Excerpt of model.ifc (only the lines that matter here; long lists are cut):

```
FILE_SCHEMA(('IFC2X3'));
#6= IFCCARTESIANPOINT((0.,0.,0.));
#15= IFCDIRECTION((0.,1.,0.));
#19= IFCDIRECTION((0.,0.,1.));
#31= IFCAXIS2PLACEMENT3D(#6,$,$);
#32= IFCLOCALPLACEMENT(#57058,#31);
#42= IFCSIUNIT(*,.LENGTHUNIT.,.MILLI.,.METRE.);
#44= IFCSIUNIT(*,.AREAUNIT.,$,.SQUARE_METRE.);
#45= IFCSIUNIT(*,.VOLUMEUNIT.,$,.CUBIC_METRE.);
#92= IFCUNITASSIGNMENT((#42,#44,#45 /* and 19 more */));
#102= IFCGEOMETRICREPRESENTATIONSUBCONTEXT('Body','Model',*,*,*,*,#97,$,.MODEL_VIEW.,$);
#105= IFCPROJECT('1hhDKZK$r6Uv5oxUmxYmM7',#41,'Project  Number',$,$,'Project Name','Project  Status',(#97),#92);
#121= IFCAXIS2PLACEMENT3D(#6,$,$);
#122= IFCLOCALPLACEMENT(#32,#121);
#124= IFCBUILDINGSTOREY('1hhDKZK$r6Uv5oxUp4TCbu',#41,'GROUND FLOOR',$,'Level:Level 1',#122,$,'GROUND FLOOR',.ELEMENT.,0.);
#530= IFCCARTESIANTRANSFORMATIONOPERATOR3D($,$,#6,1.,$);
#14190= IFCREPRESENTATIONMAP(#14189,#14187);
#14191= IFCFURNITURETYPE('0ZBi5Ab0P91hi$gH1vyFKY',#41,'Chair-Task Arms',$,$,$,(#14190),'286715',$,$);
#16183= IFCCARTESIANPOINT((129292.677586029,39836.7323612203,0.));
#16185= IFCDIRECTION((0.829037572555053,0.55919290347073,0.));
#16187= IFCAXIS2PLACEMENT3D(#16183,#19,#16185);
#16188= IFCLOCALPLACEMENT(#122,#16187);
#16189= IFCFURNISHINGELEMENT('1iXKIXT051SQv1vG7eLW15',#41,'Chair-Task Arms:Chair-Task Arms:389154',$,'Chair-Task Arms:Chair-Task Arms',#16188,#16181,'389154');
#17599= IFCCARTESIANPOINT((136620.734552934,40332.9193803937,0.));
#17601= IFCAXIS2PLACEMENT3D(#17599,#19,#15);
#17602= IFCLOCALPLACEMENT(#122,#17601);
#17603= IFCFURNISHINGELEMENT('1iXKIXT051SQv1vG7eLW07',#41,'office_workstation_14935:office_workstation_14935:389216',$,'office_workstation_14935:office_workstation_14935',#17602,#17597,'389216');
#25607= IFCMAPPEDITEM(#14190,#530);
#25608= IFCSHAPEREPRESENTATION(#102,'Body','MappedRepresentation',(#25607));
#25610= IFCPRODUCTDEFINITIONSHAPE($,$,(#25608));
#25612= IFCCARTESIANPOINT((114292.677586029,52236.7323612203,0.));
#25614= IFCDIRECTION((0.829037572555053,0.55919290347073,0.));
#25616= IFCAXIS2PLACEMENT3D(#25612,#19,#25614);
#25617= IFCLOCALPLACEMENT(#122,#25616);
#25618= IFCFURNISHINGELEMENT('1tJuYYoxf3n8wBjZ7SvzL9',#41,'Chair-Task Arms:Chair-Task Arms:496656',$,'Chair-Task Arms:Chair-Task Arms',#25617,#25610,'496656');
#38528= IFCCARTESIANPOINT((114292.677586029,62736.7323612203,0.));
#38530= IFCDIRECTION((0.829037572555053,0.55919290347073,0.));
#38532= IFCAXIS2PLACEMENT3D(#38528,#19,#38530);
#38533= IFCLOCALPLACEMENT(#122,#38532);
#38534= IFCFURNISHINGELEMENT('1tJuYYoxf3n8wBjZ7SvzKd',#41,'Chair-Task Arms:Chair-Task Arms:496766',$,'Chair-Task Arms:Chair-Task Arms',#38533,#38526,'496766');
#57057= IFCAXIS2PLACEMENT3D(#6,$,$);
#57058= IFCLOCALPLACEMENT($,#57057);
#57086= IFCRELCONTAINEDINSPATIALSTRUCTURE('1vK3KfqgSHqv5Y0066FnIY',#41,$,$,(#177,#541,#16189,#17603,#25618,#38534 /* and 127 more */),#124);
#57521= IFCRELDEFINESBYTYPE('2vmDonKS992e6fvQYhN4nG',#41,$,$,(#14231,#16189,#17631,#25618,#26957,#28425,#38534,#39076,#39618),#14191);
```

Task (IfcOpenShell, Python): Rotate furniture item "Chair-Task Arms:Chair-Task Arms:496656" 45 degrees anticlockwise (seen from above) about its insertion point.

```python
import ifcopenshell
import ifcopenshell.api.geometry
import ifcopenshell.util.placement

model = ifcopenshell.open("model.ifc")

item = model.by_guid("1tJuYYoxf3n8wBjZ7SvzL9")
matrix = ifcopenshell.util.placement.get_local_placement(item.ObjectPlacement)
matrix = matrix @ ifcopenshell.util.placement.rotation(45, "Z")
ifcopenshell.api.geometry.edit_object_placement(model, product=item, matrix=matrix, is_si=False)

print(ifcopenshell.util.placement.get_local_placement(item.ObjectPlacement).round(3) + 0.0)

model.write("model_updated.ifc")
```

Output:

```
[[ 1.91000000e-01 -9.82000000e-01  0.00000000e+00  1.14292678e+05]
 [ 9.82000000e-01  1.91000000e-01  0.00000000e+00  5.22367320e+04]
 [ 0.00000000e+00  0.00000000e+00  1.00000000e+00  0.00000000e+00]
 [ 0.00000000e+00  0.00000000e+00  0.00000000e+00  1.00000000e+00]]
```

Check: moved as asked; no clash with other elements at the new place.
